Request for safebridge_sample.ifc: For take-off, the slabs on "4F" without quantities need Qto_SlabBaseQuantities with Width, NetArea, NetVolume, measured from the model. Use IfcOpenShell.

First a look at what the model holds.

```python
import ifcopenshell
import ifcopenshell.util.element
import ifcopenshell.util.unit

model = ifcopenshell.open("safebridge_sample.ifc")
print(model.schema)
for unit_type in ("LENGTHUNIT", "AREAUNIT", "VOLUMEUNIT"):
    print(unit_type, ifcopenshell.util.unit.calculate_unit_scale(model, unit_type))
storey = next(s for s in model.by_type("IfcBuildingStorey") if s.Name == "4F")
slabs = [e for e in ifcopenshell.util.element.get_decomposition(storey) if e.is_a("IfcSlab")]
for e in sorted(slabs, key=lambda e: e.id()):
    print(e.id(), e.is_a(), e.Name, list(ifcopenshell.util.element.get_psets(e, qtos_only=True)), sep=" | ")
```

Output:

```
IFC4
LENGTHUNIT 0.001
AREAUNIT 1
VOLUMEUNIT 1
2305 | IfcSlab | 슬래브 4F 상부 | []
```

```python
import ifcopenshell
import ifcopenshell.api.pset
import ifcopenshell.geom
import ifcopenshell.util.element
import ifcopenshell.util.shape
import ifcopenshell.util.unit

model = ifcopenshell.open("safebridge_sample.ifc")
unit_scale = ifcopenshell.util.unit.calculate_unit_scale(model)
area_scale = ifcopenshell.util.unit.calculate_unit_scale(model, "AREAUNIT")
volume_scale = ifcopenshell.util.unit.calculate_unit_scale(model, "VOLUMEUNIT")
settings = ifcopenshell.geom.settings()

storey = next(s for s in model.by_type("IfcBuildingStorey") if s.Name == "4F")
slabs = [e for e in ifcopenshell.util.element.get_decomposition(storey) if e.is_a("IfcSlab")]

for e in sorted(slabs, key=lambda e: e.id()):
    if ifcopenshell.util.element.get_psets(e, qtos_only=True, should_inherit=False):
        continue
    # Geometry comes back in metres, in the element's own axes.
    shape = ifcopenshell.geom.create_shape(settings, e)
    values = {
        "Width": ifcopenshell.util.shape.get_z(shape.geometry) / unit_scale,
        "NetArea": ifcopenshell.util.shape.get_footprint_area(shape.geometry) / area_scale,
        "NetVolume": ifcopenshell.util.shape.get_volume(shape.geometry) / volume_scale,
    }
    qto = ifcopenshell.api.pset.add_qto(model, product=e, name="Qto_SlabBaseQuantities")
    ifcopenshell.api.pset.edit_qto(model, qto=qto, properties=values)
    print(e.id(), {k: round(v, 3) for k, v in values.items()})

model.write("safebridge_sample_edited.ifc")
```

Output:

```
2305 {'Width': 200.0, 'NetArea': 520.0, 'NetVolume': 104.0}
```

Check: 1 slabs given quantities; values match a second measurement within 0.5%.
